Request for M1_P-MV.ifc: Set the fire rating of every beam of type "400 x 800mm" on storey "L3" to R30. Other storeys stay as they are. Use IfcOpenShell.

First a look at what the model holds.

```python
import ifcopenshell
import ifcopenshell.util.element

model = ifcopenshell.open("M1_P-MV.ifc")
print(model.schema)
storey = next(s for s in model.by_type("IfcBuildingStorey") if s.Name == "L3")
beams = [e for e in ifcopenshell.util.element.get_decomposition(storey) if e.is_a("IfcBeam")]
seen = {}
for e in beams:
    element_type = ifcopenshell.util.element.get_type(e)
    key = (element_type.Name if element_type != e and element_type else None, ifcopenshell.util.element.get_pset(e, "Pset_BeamCommon", "FireRating"))
    seen[key] = seen.get(key, 0) + 1
for (name, value), count in sorted(seen.items(), key=str):
    print(count, "x", name, "|", value)
```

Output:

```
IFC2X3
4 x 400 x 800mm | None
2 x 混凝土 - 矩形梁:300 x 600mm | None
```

```python
import ifcopenshell
import ifcopenshell.api.pset
import ifcopenshell.util.element

model = ifcopenshell.open("M1_P-MV.ifc")

storey = next(s for s in model.by_type("IfcBuildingStorey") if s.Name == "L3")
beams = [e for e in ifcopenshell.util.element.get_decomposition(storey) if e.is_a("IfcBeam")]

count = 0
for e in beams:
    element_type = ifcopenshell.util.element.get_type(e)
    if element_type in (None, e) or element_type.Name != "400 x 800mm":
        continue
    # add_pset returns the element's existing set when there is one.
    pset = ifcopenshell.api.pset.add_pset(model, product=e, name="Pset_BeamCommon")
    ifcopenshell.api.pset.edit_pset(model, pset=pset, properties={"FireRating": "R30"})
    count += 1

print(count, "beams updated")

model.write("M1_P-MV_updated.ifc")
```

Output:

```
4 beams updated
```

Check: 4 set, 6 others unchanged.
